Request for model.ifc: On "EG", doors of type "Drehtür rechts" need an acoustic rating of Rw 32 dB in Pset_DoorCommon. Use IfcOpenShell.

First a look at what the model holds.

```python
import ifcopenshell
import ifcopenshell.util.element

model = ifcopenshell.open("model.ifc")
print(model.schema)
storey = next(s for s in model.by_type("IfcBuildingStorey") if s.Name == "EG")
doors = [e for e in ifcopenshell.util.element.get_decomposition(storey) if e.is_a("IfcDoor")]
seen = {}
for e in doors:
    element_type = ifcopenshell.util.element.get_type(e)
    key = (element_type.Name if element_type != e and element_type else None, ifcopenshell.util.element.get_pset(e, "Pset_DoorCommon", "AcousticRating"))
    seen[key] = seen.get(key, 0) + 1
for (name, value), count in sorted(seen.items(), key=str):
    print(count, "x", name, "|", value)
```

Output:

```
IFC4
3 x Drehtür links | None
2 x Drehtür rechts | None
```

```python
import ifcopenshell
import ifcopenshell.api.pset
import ifcopenshell.util.element

model = ifcopenshell.open("model.ifc")

storey = next(s for s in model.by_type("IfcBuildingStorey") if s.Name == "EG")
doors = [e for e in ifcopenshell.util.element.get_decomposition(storey) if e.is_a("IfcDoor")]

count = 0
for e in doors:
    element_type = ifcopenshell.util.element.get_type(e)
    if element_type in (None, e) or element_type.Name != "Drehtür rechts":
        continue
    # add_pset returns the element's existing set when there is one.
    pset = ifcopenshell.api.pset.add_pset(model, product=e, name="Pset_DoorCommon")
    ifcopenshell.api.pset.edit_pset(model, pset=pset, properties={"AcousticRating": "Rw 32 dB"})
    count += 1

print(count, "doors updated")

model.write("model_updated.ifc")
```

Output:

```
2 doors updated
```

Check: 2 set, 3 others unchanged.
